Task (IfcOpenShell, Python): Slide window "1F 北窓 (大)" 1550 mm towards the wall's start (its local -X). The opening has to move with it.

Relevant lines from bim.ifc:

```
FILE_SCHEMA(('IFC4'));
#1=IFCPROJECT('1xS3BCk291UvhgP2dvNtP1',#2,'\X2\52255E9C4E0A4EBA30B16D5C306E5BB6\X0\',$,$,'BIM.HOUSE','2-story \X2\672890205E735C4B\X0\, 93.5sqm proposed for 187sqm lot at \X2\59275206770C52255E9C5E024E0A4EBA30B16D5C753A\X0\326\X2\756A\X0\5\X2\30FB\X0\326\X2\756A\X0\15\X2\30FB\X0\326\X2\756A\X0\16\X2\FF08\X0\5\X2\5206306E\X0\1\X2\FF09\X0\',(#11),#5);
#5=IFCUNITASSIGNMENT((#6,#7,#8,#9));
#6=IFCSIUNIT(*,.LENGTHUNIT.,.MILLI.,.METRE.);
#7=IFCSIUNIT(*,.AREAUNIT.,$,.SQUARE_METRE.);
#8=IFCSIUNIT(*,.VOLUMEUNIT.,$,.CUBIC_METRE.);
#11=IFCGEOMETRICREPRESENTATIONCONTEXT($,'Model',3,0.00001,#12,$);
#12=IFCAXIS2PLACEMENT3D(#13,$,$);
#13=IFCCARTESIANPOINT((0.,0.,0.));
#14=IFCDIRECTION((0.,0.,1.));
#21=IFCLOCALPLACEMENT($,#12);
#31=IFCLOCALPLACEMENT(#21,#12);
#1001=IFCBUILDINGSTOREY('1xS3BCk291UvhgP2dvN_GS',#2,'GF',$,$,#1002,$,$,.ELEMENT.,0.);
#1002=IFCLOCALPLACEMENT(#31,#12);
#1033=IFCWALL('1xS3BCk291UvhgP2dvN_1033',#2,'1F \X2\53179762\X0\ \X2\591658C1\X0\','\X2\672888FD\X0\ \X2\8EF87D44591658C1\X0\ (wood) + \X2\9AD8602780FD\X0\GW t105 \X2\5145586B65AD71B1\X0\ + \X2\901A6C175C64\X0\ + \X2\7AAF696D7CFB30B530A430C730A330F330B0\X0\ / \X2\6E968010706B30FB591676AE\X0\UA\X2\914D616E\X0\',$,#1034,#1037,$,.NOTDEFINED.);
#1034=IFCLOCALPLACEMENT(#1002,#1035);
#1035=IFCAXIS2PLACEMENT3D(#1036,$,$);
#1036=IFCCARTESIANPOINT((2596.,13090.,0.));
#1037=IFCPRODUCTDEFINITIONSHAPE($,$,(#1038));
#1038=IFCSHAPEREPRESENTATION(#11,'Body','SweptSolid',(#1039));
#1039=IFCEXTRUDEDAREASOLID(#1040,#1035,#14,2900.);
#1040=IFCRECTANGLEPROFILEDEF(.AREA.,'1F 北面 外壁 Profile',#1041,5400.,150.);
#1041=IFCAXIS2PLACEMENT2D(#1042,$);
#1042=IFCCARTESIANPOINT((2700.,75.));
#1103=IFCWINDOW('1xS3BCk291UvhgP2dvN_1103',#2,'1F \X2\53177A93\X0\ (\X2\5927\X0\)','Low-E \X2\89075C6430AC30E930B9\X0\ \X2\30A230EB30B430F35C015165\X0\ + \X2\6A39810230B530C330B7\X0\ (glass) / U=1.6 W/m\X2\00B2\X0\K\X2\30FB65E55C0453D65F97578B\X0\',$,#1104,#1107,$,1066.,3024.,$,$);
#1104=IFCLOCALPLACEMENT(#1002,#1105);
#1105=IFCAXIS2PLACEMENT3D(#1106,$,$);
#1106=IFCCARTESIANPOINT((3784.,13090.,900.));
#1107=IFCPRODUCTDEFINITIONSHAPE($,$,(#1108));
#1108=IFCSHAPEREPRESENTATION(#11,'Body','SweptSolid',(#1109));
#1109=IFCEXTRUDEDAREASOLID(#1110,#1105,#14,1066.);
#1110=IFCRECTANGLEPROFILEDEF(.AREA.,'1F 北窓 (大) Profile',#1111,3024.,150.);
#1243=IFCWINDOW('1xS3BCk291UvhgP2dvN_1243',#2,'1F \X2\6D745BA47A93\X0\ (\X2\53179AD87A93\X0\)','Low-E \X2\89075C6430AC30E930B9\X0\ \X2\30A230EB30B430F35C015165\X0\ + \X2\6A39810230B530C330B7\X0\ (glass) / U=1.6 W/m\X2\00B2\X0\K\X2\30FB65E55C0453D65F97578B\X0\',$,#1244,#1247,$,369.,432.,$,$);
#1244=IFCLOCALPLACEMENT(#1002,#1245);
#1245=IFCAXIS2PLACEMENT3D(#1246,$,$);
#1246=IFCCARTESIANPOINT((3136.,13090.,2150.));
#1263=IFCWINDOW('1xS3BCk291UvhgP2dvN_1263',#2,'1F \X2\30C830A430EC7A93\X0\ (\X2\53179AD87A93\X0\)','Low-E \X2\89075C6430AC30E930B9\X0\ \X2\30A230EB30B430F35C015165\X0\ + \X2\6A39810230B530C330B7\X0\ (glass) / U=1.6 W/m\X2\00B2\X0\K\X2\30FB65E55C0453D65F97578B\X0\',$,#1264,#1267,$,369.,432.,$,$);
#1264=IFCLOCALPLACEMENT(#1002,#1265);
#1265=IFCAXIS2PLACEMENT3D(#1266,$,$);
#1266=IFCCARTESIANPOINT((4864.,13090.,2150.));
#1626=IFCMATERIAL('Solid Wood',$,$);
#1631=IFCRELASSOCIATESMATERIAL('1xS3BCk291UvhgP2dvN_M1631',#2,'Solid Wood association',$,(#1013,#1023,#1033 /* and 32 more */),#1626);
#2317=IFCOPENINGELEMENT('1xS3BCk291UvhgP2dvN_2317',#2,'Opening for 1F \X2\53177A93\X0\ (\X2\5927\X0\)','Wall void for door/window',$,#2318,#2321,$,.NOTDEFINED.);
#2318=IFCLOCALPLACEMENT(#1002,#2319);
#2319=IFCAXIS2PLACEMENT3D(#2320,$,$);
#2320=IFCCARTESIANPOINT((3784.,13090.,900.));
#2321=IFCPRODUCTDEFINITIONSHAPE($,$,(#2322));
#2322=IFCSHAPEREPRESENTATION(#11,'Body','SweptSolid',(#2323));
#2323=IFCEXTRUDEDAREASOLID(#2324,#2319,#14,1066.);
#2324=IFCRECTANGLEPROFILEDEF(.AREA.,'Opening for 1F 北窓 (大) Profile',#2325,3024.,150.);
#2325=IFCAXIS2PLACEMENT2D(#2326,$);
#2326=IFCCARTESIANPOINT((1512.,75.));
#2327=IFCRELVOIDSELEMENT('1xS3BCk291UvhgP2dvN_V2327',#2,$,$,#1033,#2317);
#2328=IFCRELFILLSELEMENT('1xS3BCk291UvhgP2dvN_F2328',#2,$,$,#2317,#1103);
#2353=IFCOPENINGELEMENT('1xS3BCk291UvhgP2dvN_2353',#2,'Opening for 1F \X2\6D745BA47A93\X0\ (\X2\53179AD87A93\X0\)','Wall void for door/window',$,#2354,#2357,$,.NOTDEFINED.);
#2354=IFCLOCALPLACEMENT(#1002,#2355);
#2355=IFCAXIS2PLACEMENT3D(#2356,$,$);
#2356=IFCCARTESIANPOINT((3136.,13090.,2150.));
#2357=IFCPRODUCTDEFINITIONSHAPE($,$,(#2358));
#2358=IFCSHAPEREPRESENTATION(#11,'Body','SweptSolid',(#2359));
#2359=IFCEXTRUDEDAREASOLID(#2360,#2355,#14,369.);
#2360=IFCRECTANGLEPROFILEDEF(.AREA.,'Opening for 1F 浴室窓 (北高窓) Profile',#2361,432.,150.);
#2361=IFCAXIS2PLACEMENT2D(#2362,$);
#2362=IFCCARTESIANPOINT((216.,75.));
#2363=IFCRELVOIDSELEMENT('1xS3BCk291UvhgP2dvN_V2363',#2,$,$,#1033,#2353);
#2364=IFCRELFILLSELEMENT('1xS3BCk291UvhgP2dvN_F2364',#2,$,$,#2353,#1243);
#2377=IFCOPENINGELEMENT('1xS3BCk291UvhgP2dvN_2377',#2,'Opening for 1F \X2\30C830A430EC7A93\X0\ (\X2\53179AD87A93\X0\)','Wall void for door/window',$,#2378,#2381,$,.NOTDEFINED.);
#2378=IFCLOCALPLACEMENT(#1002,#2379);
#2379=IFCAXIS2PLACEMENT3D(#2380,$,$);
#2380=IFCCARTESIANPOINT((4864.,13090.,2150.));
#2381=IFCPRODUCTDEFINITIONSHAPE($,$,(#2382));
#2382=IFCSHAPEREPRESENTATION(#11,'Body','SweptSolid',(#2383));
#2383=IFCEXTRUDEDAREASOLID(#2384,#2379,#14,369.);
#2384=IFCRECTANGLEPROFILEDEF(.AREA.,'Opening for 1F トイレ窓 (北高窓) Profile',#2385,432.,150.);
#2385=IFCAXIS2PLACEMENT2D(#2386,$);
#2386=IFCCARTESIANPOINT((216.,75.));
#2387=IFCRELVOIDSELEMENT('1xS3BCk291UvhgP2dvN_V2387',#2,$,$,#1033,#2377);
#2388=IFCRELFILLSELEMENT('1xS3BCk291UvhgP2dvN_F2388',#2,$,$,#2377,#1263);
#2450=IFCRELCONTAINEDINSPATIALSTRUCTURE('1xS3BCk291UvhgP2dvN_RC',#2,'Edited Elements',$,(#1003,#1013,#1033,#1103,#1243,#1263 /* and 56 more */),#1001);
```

```python
import ifcopenshell
import ifcopenshell.api.geometry
import ifcopenshell.util.placement

model = ifcopenshell.open("bim.ifc")

window = model.by_id(1103)
opening = window.FillsVoids[0].RelatingOpeningElement
wall = opening.VoidsElements[0].RelatingBuildingElement

wall_matrix = ifcopenshell.util.placement.get_local_placement(wall.ObjectPlacement)
shift = wall_matrix[:3, 0] * -1550.0
before = ifcopenshell.util.placement.get_local_placement(window.ObjectPlacement)[:3, 3].copy()

# The window is not placed relative to its opening, so move both.
for product in (opening, window):
    matrix = ifcopenshell.util.placement.get_local_placement(product.ObjectPlacement)
    matrix[:3, 3] += shift
    ifcopenshell.api.geometry.edit_object_placement(model, product=product, matrix=matrix, is_si=False)

after = ifcopenshell.util.placement.get_local_placement(window.ObjectPlacement)[:3, 3]
print("window moved by", (after - before).round(3) + 0.0)

model.write("bim_edited.ifc")
```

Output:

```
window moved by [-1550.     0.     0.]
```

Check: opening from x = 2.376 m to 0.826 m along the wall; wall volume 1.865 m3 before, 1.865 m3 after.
